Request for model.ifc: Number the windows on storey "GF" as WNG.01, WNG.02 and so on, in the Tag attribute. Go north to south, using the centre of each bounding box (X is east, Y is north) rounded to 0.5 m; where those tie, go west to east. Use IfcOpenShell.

First a look at what the model holds.

```python
import ifcopenshell
import ifcopenshell.util.element
import ifcopenshell.util.placement

model = ifcopenshell.open("model.ifc")
print(model.schema)
storey = next(s for s in model.by_type("IfcBuildingStorey") if s.Name == "GF")
windows = [e for e in ifcopenshell.util.element.get_decomposition(storey) if e.is_a("IfcWindow")]
for e in sorted(windows, key=lambda e: e.id()):
    origin = ifcopenshell.util.placement.get_local_placement(e.ObjectPlacement)[:3, 3]
    print(e.id(), e.Tag, e.Name, origin.round(2) + 0.0, sep=" | ")
```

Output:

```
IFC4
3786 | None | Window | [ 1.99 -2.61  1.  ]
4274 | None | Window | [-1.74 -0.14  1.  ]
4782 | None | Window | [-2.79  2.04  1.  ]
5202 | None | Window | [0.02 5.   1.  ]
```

```python
import ifcopenshell
import ifcopenshell.geom
import ifcopenshell.util.element
import ifcopenshell.util.shape

model = ifcopenshell.open("model.ifc")
settings = ifcopenshell.geom.settings()
settings.set("use-world-coords", True)


def centre(element):
    shape = ifcopenshell.geom.create_shape(settings, element)
    return ifcopenshell.util.shape.get_bbox_centroid(shape.geometry)


storey = next(s for s in model.by_type("IfcBuildingStorey") if s.Name == "GF")
windows = [e for e in ifcopenshell.util.element.get_decomposition(storey) if e.is_a("IfcWindow")]

# Insertion points can sit at a corner or the storey origin, so sort by the geometry (in metres).
centres = {e: centre(e) for e in windows}
windows.sort(key=lambda e: (-round(centres[e][1] / 0.5), centres[e][0]))

for i, e in enumerate(windows, start=1):
    number = f"WNG.{i:02d}"
    e.Tag = number
    print(e.id(), number)

model.write("model-out.ifc")
```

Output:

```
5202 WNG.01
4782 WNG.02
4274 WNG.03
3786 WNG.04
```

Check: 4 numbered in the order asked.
